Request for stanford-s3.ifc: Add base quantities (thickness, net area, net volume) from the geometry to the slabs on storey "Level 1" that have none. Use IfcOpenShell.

First a look at what the model holds.

```python
import ifcopenshell
import ifcopenshell.util.element
import ifcopenshell.util.unit

model = ifcopenshell.open("stanford-s3.ifc")
print(model.schema)
for unit_type in ("LENGTHUNIT", "AREAUNIT", "VOLUMEUNIT"):
    print(unit_type, ifcopenshell.util.unit.calculate_unit_scale(model, unit_type))
storey = next(s for s in model.by_type("IfcBuildingStorey") if s.Name == "Level 1")
slabs = [e for e in ifcopenshell.util.element.get_decomposition(storey) if e.is_a("IfcSlab")]
for e in sorted(slabs, key=lambda e: e.id()):
    print(e.id(), e.is_a(), e.Name, list(ifcopenshell.util.element.get_psets(e, qtos_only=True)), sep=" | ")
```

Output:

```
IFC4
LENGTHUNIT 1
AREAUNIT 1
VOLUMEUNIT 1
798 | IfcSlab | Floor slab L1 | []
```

```python
import ifcopenshell
import ifcopenshell.api.pset
import ifcopenshell.geom
import ifcopenshell.util.element
import ifcopenshell.util.shape
import ifcopenshell.util.unit

model = ifcopenshell.open("stanford-s3.ifc")
unit_scale = ifcopenshell.util.unit.calculate_unit_scale(model)
area_scale = ifcopenshell.util.unit.calculate_unit_scale(model, "AREAUNIT")
volume_scale = ifcopenshell.util.unit.calculate_unit_scale(model, "VOLUMEUNIT")
settings = ifcopenshell.geom.settings()

storey = next(s for s in model.by_type("IfcBuildingStorey") if s.Name == "Level 1")
slabs = [e for e in ifcopenshell.util.element.get_decomposition(storey) if e.is_a("IfcSlab")]

for e in sorted(slabs, key=lambda e: e.id()):
    if ifcopenshell.util.element.get_psets(e, qtos_only=True, should_inherit=False):
        continue
    # Geometry comes back in metres, in the element's own axes.
    shape = ifcopenshell.geom.create_shape(settings, e)
    values = {
        "Width": ifcopenshell.util.shape.get_z(shape.geometry) / unit_scale,
        "NetArea": ifcopenshell.util.shape.get_footprint_area(shape.geometry) / area_scale,
        "NetVolume": ifcopenshell.util.shape.get_volume(shape.geometry) / volume_scale,
    }
    qto = ifcopenshell.api.pset.add_qto(model, product=e, name="Qto_SlabBaseQuantities")
    ifcopenshell.api.pset.edit_qto(model, qto=qto, properties=values)
    print(e.id(), {k: round(v, 3) for k, v in values.items()})

model.write("stanford-s3_edited.ifc")
```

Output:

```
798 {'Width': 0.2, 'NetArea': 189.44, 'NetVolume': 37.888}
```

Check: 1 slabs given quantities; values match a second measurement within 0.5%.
